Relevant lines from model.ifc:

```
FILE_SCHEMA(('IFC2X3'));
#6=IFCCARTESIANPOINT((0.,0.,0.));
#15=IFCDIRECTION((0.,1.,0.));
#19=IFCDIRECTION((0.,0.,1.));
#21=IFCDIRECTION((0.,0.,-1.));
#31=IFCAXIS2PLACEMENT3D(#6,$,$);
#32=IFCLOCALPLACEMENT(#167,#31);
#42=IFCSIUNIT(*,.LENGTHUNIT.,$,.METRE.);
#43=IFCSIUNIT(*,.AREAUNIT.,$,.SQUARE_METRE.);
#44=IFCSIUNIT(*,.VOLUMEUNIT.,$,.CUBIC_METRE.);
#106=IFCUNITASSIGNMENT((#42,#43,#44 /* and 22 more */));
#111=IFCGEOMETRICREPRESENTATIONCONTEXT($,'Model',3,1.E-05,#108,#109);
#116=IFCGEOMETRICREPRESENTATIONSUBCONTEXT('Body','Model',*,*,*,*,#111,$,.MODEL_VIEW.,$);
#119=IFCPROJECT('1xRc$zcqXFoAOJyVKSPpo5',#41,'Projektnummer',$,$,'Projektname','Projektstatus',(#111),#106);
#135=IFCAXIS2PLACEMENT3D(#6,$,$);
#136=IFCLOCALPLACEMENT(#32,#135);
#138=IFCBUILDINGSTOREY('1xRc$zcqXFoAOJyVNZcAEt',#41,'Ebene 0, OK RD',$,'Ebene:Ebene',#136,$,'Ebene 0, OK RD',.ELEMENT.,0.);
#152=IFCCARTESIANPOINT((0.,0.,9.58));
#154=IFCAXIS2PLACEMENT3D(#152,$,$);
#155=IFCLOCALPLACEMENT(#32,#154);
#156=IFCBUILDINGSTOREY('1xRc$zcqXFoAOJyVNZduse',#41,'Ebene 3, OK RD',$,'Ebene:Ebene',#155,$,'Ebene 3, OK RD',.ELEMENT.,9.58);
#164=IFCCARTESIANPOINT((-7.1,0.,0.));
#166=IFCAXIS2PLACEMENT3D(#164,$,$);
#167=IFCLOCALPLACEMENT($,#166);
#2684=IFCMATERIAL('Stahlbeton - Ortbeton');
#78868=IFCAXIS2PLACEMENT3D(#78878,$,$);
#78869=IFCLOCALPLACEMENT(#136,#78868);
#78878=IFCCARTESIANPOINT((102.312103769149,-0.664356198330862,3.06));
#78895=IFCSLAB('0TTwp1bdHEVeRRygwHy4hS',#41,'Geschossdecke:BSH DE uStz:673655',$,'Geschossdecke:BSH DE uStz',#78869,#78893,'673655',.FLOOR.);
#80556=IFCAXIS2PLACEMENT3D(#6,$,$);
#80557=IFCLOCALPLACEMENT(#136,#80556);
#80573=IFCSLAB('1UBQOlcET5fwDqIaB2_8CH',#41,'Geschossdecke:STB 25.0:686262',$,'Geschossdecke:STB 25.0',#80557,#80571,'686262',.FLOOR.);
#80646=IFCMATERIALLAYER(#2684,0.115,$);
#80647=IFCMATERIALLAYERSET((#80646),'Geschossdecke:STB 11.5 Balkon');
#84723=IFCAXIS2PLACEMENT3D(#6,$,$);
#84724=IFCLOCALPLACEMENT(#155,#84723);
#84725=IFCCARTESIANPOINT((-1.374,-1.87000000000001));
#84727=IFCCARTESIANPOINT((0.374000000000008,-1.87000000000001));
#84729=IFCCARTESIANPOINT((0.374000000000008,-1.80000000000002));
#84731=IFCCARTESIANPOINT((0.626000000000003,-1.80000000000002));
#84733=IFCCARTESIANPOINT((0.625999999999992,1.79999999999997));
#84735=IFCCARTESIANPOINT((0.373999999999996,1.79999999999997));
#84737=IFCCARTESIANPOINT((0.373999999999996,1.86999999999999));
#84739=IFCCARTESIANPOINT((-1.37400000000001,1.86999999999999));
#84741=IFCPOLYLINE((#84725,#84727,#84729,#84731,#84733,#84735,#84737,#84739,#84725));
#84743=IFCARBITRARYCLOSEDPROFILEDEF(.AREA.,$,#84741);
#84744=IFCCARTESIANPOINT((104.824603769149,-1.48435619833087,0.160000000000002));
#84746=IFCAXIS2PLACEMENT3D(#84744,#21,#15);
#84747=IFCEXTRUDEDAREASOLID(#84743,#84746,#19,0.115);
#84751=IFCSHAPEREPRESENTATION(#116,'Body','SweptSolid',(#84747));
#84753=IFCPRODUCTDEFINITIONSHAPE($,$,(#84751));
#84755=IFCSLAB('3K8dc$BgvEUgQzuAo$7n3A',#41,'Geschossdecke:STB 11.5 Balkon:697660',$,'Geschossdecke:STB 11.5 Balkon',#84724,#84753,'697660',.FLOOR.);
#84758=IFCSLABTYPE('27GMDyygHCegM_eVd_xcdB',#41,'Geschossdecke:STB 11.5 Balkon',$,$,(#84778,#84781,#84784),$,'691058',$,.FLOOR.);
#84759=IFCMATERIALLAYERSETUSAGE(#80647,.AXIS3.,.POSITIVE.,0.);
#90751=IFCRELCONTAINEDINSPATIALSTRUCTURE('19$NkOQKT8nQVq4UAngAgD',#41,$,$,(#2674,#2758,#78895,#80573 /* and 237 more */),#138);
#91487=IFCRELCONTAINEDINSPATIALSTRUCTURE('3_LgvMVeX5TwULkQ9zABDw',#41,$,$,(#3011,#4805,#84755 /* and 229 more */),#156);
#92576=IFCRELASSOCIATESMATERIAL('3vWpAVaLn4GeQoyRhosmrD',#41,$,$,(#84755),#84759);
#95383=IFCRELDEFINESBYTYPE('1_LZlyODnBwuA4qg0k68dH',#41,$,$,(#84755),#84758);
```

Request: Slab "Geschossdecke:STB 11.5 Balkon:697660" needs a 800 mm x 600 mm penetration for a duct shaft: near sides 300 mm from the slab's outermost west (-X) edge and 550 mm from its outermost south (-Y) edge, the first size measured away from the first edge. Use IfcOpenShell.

```python
import numpy as np
import ifcopenshell
import ifcopenshell.api.feature
import ifcopenshell.api.geometry
import ifcopenshell.api.root
import ifcopenshell.geom
import ifcopenshell.util.placement
import ifcopenshell.util.representation
import ifcopenshell.util.shape
import ifcopenshell.util.unit

model = ifcopenshell.open("model.ifc")
unit_scale = ifcopenshell.util.unit.calculate_unit_scale(model)
settings = ifcopenshell.geom.settings()


def volume(element):
    """Net volume in cubic metres, openings subtracted."""
    shape = ifcopenshell.geom.create_shape(settings, element)
    return ifcopenshell.util.shape.get_volume(shape.geometry)


slab = model.by_guid("3K8dc$BgvEUgQzuAo$7n3A")
before = volume(slab)

# Extent in the slab's own axes, in metres. The edges named are its -X and -Y sides.
slab_shape = ifcopenshell.geom.create_shape(settings, slab)
vertices = ifcopenshell.util.shape.get_vertices(slab_shape.geometry)
x_min, y_min, bottom = vertices.min(axis=0)
top = vertices[:, 2].max()

opening = ifcopenshell.api.root.create_entity(model, ifc_class="IfcOpeningElement", name="Duct shaft opening")
context = ifcopenshell.util.representation.get_context(model, "Model", "Body", "MODEL_VIEW")
width, depth = 0.8, 0.6
outline = [(0.0, 0.0), (width, 0.0), (width, depth), (0.0, depth), (0.0, 0.0)]
# Overshoot both faces by 50 mm so the cut is clean.
shape = ifcopenshell.api.geometry.add_slab_representation(
    model, context=context, depth=top - bottom + 0.1, polyline=outline
)
ifcopenshell.api.geometry.assign_representation(model, product=opening, representation=shape)

matrix = ifcopenshell.util.placement.get_local_placement(slab.ObjectPlacement)
matrix[:, 3] = matrix @ np.append(np.array([x_min + 0.3, y_min + 0.55, bottom - 0.05]) / unit_scale, 1.0)
ifcopenshell.api.geometry.edit_object_placement(model, product=opening, matrix=matrix, is_si=False)
ifcopenshell.api.feature.add_feature(model, feature=opening, element=slab)

after = volume(slab)

print(f"slab volume {before:.3f} -> {after:.3f} m3")

model.write("model_rev.ifc")
```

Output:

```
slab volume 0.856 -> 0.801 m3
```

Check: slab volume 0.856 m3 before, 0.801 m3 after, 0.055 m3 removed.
